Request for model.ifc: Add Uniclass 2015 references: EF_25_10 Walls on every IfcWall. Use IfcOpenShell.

First a look at what the model holds.

```python
import ifcopenshell

model = ifcopenshell.open("model.ifc")
print(model.schema)
print("classifications:", [c.Name for c in model.by_type("IfcClassification")])
for ifc_class in ("IfcDoor", "IfcRoof", "IfcStair", "IfcWall", "IfcWindow"):
    print(ifc_class, len(model.by_type(ifc_class)))
```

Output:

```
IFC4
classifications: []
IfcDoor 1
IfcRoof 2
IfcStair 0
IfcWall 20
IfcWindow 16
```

```python
import ifcopenshell
import ifcopenshell.api.classification

model = ifcopenshell.open("model.ifc")

system = ifcopenshell.api.classification.add_classification(model, classification="Uniclass 2015")

codes = {
    "IfcWall": ("EF_25_10", "Walls"),
}
for ifc_class, (code, name) in codes.items():
    products = model.by_type(ifc_class)
    ifcopenshell.api.classification.add_reference(
        model, products=products, classification=system, identification=code, name=name
    )
    print(code, len(products))

model.write("model-out.ifc")
```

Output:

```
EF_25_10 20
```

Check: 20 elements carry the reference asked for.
